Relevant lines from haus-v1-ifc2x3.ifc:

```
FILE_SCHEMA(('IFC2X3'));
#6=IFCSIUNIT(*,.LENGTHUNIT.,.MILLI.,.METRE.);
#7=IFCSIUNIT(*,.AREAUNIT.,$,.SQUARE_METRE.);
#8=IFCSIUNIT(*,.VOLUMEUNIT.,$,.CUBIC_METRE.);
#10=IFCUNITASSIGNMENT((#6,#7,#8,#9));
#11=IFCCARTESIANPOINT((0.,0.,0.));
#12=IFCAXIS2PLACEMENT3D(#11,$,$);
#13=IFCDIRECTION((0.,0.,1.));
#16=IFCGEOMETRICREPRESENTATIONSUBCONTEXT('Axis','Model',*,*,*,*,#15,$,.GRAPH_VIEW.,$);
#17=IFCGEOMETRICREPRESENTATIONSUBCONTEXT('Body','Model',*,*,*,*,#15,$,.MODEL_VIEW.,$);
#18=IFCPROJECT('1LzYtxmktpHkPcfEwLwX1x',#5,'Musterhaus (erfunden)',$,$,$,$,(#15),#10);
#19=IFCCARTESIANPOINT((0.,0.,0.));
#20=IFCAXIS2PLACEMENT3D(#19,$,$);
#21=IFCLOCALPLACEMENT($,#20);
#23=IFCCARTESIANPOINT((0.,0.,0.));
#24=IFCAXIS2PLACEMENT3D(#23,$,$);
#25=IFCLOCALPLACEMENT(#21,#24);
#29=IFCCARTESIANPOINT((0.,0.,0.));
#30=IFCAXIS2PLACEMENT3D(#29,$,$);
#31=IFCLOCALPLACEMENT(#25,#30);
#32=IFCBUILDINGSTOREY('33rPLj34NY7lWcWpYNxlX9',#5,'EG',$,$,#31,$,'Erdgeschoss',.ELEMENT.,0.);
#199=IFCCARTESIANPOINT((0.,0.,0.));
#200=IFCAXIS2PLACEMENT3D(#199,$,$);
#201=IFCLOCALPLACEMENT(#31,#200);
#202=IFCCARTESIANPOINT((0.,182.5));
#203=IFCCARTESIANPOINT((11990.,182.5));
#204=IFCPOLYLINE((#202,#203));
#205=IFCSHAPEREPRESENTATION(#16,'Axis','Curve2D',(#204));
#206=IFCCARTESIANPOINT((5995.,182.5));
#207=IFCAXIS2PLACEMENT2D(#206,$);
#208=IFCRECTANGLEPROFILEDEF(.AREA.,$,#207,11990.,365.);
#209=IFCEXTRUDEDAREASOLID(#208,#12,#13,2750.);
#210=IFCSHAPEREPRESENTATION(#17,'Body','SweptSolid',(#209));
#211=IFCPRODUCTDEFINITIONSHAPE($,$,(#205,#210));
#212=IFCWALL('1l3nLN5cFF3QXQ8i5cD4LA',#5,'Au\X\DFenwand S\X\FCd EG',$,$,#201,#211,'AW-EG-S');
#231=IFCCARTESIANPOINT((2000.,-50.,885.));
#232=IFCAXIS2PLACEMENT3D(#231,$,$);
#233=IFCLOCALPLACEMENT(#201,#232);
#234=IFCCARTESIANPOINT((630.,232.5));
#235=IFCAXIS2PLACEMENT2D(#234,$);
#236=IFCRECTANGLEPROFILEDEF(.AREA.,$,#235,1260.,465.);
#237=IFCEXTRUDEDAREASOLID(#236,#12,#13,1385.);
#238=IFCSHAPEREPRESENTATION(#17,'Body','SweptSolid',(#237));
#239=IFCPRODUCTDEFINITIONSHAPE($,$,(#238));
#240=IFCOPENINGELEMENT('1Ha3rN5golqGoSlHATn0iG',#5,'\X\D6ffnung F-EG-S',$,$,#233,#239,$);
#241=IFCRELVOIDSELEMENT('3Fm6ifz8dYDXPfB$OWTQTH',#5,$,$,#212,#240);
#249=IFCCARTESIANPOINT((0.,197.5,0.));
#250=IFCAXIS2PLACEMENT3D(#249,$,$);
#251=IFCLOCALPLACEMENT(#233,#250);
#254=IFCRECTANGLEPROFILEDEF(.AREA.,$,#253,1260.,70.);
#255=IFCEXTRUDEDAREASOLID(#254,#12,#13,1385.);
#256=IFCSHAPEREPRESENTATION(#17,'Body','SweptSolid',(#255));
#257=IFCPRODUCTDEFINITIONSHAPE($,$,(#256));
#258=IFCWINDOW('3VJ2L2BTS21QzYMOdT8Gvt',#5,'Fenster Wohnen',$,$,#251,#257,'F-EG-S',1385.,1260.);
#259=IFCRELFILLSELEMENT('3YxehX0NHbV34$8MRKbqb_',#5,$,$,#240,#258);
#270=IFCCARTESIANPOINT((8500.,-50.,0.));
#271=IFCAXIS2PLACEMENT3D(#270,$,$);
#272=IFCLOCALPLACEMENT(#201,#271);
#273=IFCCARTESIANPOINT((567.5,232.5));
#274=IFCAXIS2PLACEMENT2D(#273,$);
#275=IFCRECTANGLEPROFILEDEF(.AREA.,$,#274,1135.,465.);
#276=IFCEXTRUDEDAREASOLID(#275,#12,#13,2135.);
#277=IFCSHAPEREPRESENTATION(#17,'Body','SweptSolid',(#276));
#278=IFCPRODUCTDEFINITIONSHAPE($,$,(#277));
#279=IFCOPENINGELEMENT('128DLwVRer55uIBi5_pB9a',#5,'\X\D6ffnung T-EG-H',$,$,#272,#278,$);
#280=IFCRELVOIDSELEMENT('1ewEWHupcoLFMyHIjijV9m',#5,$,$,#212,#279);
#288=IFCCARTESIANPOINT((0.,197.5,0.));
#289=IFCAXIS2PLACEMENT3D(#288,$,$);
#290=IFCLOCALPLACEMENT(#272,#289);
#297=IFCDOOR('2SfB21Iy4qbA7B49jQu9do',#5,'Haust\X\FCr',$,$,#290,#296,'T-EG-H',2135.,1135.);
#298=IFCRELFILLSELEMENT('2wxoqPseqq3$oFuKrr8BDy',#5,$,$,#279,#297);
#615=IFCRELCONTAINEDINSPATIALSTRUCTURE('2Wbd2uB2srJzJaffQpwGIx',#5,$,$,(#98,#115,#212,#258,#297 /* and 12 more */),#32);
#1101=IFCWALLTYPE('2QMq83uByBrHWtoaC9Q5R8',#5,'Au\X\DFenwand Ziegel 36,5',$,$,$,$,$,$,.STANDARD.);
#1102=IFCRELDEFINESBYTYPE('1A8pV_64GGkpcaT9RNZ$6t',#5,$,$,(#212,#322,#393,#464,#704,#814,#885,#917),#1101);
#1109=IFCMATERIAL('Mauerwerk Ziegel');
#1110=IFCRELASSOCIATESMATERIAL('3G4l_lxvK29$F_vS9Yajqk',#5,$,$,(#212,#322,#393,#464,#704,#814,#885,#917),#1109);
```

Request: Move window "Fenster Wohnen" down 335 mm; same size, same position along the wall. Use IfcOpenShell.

```python
import numpy as np
import ifcopenshell
import ifcopenshell.api.geometry
import ifcopenshell.util.placement
import ifcopenshell.util.unit

model = ifcopenshell.open("haus-v1-ifc2x3.ifc")
unit_scale = ifcopenshell.util.unit.calculate_unit_scale(model)

window = model.by_id(258)
opening = window.FillsVoids[0].RelatingOpeningElement
dz = -0.335 / unit_scale

shift = np.array([0.0, 0.0, dz])
# The window is placed relative to its opening, so it follows when the opening moves.
matrix = ifcopenshell.util.placement.get_local_placement(opening.ObjectPlacement)
matrix[:3, 3] += shift
ifcopenshell.api.geometry.edit_object_placement(
    model, product=opening, matrix=matrix, is_si=False, should_transform_children=True
)

print(f"moved by {dz * unit_scale:+.3f} m")

model.write("haus-v1-ifc2x3-out.ifc")
```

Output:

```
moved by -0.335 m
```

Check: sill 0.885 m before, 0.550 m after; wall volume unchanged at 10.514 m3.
